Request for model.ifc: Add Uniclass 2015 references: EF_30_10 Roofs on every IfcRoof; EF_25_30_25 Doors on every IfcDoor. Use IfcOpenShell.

First a look at what the model holds.

```python
import ifcopenshell

model = ifcopenshell.open("model.ifc")
print(model.schema)
print("classifications:", [c.Name for c in model.by_type("IfcClassification")])
for ifc_class in ("IfcDoor", "IfcRoof", "IfcStair", "IfcWall", "IfcWindow"):
    print(ifc_class, len(model.by_type(ifc_class)))
```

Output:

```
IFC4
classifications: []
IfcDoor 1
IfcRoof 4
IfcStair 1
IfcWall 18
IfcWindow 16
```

```python
import ifcopenshell
import ifcopenshell.api.classification

model = ifcopenshell.open("model.ifc")

system = ifcopenshell.api.classification.add_classification(model, classification="Uniclass 2015")

codes = {
    "IfcRoof": ("EF_30_10", "Roofs"),
    "IfcDoor": ("EF_25_30_25", "Doors"),
}
for ifc_class, (code, name) in codes.items():
    products = model.by_type(ifc_class)
    ifcopenshell.api.classification.add_reference(
        model, products=products, classification=system, identification=code, name=name
    )
    print(code, len(products))

model.write("model_rev.ifc")
```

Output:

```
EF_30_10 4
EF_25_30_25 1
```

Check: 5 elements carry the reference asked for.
